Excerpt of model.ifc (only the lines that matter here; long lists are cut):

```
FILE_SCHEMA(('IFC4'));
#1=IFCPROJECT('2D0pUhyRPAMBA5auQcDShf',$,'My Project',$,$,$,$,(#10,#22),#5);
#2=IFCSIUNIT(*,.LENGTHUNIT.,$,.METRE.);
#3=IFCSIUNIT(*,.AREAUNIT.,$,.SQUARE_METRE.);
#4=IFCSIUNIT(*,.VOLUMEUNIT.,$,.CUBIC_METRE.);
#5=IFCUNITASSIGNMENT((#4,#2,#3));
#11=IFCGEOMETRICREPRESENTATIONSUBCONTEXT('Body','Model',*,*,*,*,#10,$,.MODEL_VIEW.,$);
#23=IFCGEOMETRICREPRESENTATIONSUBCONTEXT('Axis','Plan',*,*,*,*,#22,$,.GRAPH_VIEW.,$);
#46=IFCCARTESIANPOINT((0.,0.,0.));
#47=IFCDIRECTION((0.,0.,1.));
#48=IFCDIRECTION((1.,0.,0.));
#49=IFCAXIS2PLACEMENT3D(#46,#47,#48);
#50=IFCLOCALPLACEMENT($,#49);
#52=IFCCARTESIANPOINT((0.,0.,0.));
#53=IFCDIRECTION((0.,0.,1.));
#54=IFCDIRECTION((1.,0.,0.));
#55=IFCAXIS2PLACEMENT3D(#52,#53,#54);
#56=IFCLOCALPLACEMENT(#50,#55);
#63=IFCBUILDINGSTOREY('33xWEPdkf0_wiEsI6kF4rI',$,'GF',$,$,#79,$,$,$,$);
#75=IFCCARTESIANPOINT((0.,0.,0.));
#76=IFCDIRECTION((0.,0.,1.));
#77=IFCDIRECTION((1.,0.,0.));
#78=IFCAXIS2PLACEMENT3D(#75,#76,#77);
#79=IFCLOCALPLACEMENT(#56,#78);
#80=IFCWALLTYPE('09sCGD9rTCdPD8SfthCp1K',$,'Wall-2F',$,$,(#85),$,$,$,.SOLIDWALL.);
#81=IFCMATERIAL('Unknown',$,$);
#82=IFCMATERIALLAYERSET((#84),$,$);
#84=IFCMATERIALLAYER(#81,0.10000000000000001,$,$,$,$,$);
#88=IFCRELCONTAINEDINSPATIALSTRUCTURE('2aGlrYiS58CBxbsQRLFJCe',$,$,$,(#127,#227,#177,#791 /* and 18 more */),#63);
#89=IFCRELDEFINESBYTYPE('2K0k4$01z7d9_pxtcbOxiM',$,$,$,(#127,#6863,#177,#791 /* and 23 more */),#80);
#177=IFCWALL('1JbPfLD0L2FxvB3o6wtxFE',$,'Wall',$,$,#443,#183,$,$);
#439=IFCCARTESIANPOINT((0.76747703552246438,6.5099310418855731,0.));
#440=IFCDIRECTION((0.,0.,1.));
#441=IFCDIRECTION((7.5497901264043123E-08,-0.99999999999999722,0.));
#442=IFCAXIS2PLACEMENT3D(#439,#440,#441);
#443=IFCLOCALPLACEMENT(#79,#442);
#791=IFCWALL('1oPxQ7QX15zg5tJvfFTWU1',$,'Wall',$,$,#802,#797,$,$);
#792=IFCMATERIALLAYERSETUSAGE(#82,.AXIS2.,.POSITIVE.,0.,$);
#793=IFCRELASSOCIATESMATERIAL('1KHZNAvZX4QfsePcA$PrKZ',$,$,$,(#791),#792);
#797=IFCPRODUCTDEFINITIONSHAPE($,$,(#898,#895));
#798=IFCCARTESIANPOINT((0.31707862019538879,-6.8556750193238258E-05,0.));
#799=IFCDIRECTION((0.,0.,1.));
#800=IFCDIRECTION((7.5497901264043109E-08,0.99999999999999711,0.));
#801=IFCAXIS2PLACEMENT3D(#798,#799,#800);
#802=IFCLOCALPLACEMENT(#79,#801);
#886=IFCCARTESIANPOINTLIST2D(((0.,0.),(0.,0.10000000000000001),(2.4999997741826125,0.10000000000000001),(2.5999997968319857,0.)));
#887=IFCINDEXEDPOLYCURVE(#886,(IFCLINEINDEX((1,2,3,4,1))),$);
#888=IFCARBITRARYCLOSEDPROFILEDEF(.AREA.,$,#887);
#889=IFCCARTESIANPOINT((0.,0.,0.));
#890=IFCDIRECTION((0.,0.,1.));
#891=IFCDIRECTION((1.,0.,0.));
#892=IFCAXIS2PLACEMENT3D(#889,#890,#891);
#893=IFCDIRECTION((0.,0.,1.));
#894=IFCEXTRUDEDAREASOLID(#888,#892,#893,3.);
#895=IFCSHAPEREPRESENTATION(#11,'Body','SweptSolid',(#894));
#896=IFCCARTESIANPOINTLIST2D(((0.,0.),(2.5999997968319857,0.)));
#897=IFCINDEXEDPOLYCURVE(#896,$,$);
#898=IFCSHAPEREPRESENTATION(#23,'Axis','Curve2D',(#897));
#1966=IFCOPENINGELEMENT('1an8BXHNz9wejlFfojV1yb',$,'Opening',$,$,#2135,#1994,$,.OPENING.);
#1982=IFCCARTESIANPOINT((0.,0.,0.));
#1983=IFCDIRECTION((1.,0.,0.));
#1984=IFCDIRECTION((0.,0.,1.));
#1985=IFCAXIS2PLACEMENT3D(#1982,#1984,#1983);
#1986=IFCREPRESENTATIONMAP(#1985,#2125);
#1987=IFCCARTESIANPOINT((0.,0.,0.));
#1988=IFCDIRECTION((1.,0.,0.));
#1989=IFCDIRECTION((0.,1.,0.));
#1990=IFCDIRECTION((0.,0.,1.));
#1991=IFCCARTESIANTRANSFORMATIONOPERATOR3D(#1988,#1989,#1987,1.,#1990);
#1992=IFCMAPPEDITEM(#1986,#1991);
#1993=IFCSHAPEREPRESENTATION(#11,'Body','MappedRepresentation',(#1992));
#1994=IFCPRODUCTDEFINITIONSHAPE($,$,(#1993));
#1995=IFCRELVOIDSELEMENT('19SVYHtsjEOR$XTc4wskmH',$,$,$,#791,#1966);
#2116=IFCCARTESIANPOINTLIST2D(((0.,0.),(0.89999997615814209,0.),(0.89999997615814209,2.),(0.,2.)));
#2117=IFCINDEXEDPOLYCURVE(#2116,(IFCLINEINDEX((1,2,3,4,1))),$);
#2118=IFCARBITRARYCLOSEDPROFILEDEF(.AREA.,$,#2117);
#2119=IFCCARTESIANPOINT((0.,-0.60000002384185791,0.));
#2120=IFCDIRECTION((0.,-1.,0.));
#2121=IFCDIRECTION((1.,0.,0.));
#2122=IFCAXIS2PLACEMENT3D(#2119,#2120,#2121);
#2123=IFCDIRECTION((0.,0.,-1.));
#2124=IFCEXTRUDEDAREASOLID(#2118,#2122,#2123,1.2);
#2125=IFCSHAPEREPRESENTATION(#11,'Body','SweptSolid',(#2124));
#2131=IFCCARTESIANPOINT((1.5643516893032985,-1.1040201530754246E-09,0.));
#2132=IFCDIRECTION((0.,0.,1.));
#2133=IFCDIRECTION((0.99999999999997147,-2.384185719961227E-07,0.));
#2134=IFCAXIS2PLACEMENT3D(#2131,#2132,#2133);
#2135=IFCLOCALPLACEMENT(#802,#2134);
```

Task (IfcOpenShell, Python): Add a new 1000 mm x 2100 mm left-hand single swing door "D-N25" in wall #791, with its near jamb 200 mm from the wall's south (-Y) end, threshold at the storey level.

```python
import numpy as np
import ifcopenshell
import ifcopenshell.api.feature
import ifcopenshell.api.geometry
import ifcopenshell.api.root
import ifcopenshell.api.spatial
import ifcopenshell.geom
import ifcopenshell.util.element
import ifcopenshell.util.placement
import ifcopenshell.util.representation
import ifcopenshell.util.shape
import ifcopenshell.util.unit

model = ifcopenshell.open("model.ifc")
unit_scale = ifcopenshell.util.unit.calculate_unit_scale(model)
settings = ifcopenshell.geom.settings()


def volume(element):
    """Net volume in cubic metres, openings subtracted."""
    shape = ifcopenshell.geom.create_shape(settings, element)
    return ifcopenshell.util.shape.get_volume(shape.geometry)


wall = model.by_guid("1oPxQ7QX15zg5tJvfFTWU1")
storey = ifcopenshell.util.element.get_container(wall, ifc_class="IfcBuildingStorey")
context = ifcopenshell.util.representation.get_context(model, "Model", "Body", "MODEL_VIEW")
before = volume(wall)

width, height, from_end, sill = 1, 2.1, 0.2, 0.0  # metres

# The wall runs along its own X axis, and the end named is its -X end.
wall_shape = ifcopenshell.geom.create_shape(settings, wall)
x, y, z = ifcopenshell.util.shape.get_vertices(wall_shape.geometry).T
start = x.min() + from_end
face, thickness = float(y.min()), float(y.max() - y.min())
wall_matrix = ifcopenshell.util.placement.get_local_placement(wall.ObjectPlacement)
level = ifcopenshell.util.placement.get_local_placement(storey.ObjectPlacement)[2, 3]


def in_wall(x, y):
    """Placement at x, y metres in the wall's axes, at sill height."""
    matrix = wall_matrix.copy()
    matrix[:, 3] = wall_matrix @ np.array([x / unit_scale, y / unit_scale, 0.0, 1.0])
    matrix[2, 3] = level + sill / unit_scale
    return matrix


# Opening: a box that overshoots both wall faces by 50 mm.
opening = ifcopenshell.api.root.create_entity(model, ifc_class="IfcOpeningElement", predefined_type="OPENING")
box = ifcopenshell.api.geometry.add_wall_representation(
    model, context=context, length=width, height=height, thickness=thickness + 0.1
)
ifcopenshell.api.geometry.assign_representation(model, product=opening, representation=box)
ifcopenshell.api.geometry.edit_object_placement(model, product=opening, matrix=in_wall(start, face - 0.05), is_si=False)
ifcopenshell.api.feature.add_feature(model, feature=opening, element=wall)

door = ifcopenshell.api.root.create_entity(model, ifc_class="IfcDoor", name="D-N25", predefined_type="DOOR")
door.OverallWidth, door.OverallHeight = width / unit_scale, height / unit_scale
door.OperationType = "SINGLE_SWING_LEFT"
body = ifcopenshell.api.geometry.add_door_representation(
    model,
    context=context,
    overall_width=door.OverallWidth,
    overall_height=door.OverallHeight,
    operation_type="SINGLE_SWING_LEFT",
    lining_properties={"LiningDepth": thickness / unit_scale, "ThresholdDepth": thickness / unit_scale},
)
ifcopenshell.api.geometry.assign_representation(model, product=door, representation=body)
ifcopenshell.api.spatial.assign_container(model, products=[door], relating_structure=storey)
ifcopenshell.api.feature.add_filling(model, opening=opening, element=door)

# The lining spans the wall, so the door starts at the wall face.
ifcopenshell.api.geometry.edit_object_placement(model, product=door, matrix=in_wall(start, face), is_si=False)

after = volume(wall)

print(f"wall volume {before:.3f} -> {after:.3f} m3")

model.write("model_rev.ifc")
```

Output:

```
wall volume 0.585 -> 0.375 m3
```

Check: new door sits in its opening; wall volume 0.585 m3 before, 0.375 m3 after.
